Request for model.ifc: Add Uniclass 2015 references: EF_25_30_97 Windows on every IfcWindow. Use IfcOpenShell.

First a look at what the model holds.

```python
import ifcopenshell

model = ifcopenshell.open("model.ifc")
print(model.schema)
print("classifications:", [c.Name for c in model.by_type("IfcClassification")])
for ifc_class in ("IfcDoor", "IfcRoof", "IfcStair", "IfcWall", "IfcWindow"):
    print(ifc_class, len(model.by_type(ifc_class)))
```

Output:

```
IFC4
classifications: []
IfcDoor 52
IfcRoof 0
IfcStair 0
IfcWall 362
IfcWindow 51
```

```python
import ifcopenshell
import ifcopenshell.api.classification

model = ifcopenshell.open("model.ifc")

system = ifcopenshell.api.classification.add_classification(model, classification="Uniclass 2015")

codes = {
    "IfcWindow": ("EF_25_30_97", "Windows"),
}
for ifc_class, (code, name) in codes.items():
    products = model.by_type(ifc_class)
    ifcopenshell.api.classification.add_reference(
        model, products=products, classification=system, identification=code, name=name
    )
    print(code, len(products))

model.write("model_v2.ifc")
```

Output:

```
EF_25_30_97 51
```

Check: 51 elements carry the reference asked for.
